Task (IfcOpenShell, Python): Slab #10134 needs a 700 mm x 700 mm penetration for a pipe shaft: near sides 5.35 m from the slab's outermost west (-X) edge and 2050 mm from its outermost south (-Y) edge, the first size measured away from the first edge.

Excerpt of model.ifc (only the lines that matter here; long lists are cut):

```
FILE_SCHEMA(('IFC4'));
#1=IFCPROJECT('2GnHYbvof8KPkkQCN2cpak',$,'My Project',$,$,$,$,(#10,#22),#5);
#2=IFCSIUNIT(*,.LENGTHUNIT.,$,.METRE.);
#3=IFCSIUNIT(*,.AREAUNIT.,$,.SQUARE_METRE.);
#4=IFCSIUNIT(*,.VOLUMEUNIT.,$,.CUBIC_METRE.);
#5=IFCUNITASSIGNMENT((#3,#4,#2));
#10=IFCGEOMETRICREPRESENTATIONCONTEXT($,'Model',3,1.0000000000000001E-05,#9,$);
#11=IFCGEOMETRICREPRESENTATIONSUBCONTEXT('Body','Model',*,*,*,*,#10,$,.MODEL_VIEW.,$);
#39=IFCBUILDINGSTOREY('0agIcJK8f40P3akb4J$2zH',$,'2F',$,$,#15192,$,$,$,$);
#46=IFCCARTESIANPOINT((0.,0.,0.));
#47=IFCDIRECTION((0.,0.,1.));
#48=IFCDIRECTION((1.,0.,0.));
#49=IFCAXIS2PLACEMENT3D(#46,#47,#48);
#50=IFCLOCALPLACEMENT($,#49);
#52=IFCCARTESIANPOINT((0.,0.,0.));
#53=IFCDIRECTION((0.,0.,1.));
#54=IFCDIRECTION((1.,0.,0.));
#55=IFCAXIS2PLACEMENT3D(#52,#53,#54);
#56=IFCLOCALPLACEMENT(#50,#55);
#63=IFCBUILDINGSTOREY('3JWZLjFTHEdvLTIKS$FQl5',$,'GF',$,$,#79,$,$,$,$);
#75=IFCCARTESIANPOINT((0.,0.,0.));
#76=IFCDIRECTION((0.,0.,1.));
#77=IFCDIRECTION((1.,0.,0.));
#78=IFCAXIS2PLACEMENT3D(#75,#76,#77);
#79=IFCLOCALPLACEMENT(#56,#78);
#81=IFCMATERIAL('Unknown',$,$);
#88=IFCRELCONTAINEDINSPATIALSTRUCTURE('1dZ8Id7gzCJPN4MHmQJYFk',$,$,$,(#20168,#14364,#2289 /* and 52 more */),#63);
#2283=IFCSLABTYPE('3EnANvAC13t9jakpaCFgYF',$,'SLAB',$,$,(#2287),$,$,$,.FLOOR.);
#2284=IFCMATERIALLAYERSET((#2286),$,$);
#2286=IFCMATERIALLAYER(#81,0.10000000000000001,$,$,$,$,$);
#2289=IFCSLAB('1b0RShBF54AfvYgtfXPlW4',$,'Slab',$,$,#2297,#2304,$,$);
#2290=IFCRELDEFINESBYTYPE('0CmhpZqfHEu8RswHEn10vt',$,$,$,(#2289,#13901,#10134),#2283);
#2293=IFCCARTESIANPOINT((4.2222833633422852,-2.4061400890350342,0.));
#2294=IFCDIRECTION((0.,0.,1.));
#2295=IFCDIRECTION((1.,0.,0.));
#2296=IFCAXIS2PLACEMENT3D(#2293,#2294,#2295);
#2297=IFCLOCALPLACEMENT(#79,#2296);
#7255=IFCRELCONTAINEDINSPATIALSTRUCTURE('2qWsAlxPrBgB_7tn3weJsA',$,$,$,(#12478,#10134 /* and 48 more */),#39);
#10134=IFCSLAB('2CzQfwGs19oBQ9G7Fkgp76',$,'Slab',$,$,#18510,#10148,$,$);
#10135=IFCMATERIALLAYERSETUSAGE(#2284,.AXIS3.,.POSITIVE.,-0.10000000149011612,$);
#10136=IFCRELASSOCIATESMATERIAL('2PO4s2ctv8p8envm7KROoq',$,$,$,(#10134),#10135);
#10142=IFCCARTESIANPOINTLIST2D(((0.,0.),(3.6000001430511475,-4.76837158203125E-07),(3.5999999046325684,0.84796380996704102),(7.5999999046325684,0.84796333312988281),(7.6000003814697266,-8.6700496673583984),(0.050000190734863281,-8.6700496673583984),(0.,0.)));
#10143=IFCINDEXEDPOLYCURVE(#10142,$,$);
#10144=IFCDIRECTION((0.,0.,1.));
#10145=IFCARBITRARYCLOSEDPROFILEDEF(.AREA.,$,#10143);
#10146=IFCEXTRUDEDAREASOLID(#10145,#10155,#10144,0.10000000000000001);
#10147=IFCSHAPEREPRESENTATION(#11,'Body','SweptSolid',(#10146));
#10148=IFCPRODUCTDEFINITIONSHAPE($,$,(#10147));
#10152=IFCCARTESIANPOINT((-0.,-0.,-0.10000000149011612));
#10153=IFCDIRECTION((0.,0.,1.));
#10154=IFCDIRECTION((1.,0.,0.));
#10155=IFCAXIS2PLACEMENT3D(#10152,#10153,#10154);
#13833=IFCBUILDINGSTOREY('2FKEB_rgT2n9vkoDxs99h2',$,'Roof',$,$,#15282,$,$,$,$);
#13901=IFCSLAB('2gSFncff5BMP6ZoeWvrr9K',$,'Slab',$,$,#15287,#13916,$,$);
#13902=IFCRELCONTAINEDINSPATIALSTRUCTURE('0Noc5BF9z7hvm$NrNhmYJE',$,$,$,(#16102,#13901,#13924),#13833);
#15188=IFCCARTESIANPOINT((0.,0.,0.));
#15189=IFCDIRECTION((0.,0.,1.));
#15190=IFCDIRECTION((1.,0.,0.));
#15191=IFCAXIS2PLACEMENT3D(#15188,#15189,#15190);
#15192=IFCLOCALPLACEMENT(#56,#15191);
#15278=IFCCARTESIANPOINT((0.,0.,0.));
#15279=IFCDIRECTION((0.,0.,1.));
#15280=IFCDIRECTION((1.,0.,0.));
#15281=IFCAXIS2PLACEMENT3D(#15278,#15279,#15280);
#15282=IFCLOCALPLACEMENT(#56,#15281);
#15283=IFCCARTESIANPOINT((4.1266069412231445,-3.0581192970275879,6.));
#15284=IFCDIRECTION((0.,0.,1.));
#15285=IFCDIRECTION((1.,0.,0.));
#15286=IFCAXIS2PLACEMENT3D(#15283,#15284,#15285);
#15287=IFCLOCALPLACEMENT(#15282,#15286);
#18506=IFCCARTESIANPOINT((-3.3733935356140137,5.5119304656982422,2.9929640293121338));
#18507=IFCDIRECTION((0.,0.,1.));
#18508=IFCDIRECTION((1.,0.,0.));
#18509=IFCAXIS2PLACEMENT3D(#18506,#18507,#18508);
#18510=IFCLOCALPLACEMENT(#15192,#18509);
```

```python
import numpy as np
import ifcopenshell
import ifcopenshell.api.feature
import ifcopenshell.api.geometry
import ifcopenshell.api.root
import ifcopenshell.geom
import ifcopenshell.util.placement
import ifcopenshell.util.representation
import ifcopenshell.util.shape
import ifcopenshell.util.unit

model = ifcopenshell.open("model.ifc")
unit_scale = ifcopenshell.util.unit.calculate_unit_scale(model)
settings = ifcopenshell.geom.settings()


def volume(element):
    """Net volume in cubic metres, openings subtracted."""
    shape = ifcopenshell.geom.create_shape(settings, element)
    return ifcopenshell.util.shape.get_volume(shape.geometry)


slab = model.by_id(10134)
before = volume(slab)

# Extent in the slab's own axes, in metres. The edges named are its -X and -Y sides.
slab_shape = ifcopenshell.geom.create_shape(settings, slab)
vertices = ifcopenshell.util.shape.get_vertices(slab_shape.geometry)
x_min, y_min, bottom = vertices.min(axis=0)
top = vertices[:, 2].max()

opening = ifcopenshell.api.root.create_entity(model, ifc_class="IfcOpeningElement", name="Pipe shaft opening", predefined_type="OPENING")
context = ifcopenshell.util.representation.get_context(model, "Model", "Body", "MODEL_VIEW")
width, depth = 0.7, 0.7
outline = [(0.0, 0.0), (width, 0.0), (width, depth), (0.0, depth), (0.0, 0.0)]
# Overshoot both faces by 50 mm so the cut is clean.
shape = ifcopenshell.api.geometry.add_slab_representation(
    model, context=context, depth=top - bottom + 0.1, polyline=outline
)
ifcopenshell.api.geometry.assign_representation(model, product=opening, representation=shape)

matrix = ifcopenshell.util.placement.get_local_placement(slab.ObjectPlacement)
matrix[:, 3] = matrix @ np.append(np.array([x_min + 5.35, y_min + 2.05, bottom - 0.05]) / unit_scale, 1.0)
ifcopenshell.api.geometry.edit_object_placement(model, product=opening, matrix=matrix, is_si=False)
ifcopenshell.api.feature.add_feature(model, feature=opening, element=slab)

after = volume(slab)

print(f"slab volume {before:.3f} -> {after:.3f} m3")

model.write("model_edited.ifc")
```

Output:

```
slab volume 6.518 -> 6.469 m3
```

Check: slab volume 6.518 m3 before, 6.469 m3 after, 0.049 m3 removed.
